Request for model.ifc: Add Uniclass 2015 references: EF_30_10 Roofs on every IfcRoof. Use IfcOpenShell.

First a look at what the model holds.

```python
import ifcopenshell

model = ifcopenshell.open("model.ifc")
print(model.schema)
print("classifications:", [c.Name for c in model.by_type("IfcClassification")])
for ifc_class in ("IfcDoor", "IfcRoof", "IfcStair", "IfcWall", "IfcWindow"):
    print(ifc_class, len(model.by_type(ifc_class)))
```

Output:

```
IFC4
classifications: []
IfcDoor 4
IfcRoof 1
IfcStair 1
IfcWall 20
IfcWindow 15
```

```python
import ifcopenshell
import ifcopenshell.api.classification

model = ifcopenshell.open("model.ifc")

system = ifcopenshell.api.classification.add_classification(model, classification="Uniclass 2015")

codes = {
    "IfcRoof": ("EF_30_10", "Roofs"),
}
for ifc_class, (code, name) in codes.items():
    products = model.by_type(ifc_class)
    ifcopenshell.api.classification.add_reference(
        model, products=products, classification=system, identification=code, name=name
    )
    print(code, len(products))

model.write("model_rev.ifc")
```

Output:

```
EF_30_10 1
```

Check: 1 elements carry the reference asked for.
